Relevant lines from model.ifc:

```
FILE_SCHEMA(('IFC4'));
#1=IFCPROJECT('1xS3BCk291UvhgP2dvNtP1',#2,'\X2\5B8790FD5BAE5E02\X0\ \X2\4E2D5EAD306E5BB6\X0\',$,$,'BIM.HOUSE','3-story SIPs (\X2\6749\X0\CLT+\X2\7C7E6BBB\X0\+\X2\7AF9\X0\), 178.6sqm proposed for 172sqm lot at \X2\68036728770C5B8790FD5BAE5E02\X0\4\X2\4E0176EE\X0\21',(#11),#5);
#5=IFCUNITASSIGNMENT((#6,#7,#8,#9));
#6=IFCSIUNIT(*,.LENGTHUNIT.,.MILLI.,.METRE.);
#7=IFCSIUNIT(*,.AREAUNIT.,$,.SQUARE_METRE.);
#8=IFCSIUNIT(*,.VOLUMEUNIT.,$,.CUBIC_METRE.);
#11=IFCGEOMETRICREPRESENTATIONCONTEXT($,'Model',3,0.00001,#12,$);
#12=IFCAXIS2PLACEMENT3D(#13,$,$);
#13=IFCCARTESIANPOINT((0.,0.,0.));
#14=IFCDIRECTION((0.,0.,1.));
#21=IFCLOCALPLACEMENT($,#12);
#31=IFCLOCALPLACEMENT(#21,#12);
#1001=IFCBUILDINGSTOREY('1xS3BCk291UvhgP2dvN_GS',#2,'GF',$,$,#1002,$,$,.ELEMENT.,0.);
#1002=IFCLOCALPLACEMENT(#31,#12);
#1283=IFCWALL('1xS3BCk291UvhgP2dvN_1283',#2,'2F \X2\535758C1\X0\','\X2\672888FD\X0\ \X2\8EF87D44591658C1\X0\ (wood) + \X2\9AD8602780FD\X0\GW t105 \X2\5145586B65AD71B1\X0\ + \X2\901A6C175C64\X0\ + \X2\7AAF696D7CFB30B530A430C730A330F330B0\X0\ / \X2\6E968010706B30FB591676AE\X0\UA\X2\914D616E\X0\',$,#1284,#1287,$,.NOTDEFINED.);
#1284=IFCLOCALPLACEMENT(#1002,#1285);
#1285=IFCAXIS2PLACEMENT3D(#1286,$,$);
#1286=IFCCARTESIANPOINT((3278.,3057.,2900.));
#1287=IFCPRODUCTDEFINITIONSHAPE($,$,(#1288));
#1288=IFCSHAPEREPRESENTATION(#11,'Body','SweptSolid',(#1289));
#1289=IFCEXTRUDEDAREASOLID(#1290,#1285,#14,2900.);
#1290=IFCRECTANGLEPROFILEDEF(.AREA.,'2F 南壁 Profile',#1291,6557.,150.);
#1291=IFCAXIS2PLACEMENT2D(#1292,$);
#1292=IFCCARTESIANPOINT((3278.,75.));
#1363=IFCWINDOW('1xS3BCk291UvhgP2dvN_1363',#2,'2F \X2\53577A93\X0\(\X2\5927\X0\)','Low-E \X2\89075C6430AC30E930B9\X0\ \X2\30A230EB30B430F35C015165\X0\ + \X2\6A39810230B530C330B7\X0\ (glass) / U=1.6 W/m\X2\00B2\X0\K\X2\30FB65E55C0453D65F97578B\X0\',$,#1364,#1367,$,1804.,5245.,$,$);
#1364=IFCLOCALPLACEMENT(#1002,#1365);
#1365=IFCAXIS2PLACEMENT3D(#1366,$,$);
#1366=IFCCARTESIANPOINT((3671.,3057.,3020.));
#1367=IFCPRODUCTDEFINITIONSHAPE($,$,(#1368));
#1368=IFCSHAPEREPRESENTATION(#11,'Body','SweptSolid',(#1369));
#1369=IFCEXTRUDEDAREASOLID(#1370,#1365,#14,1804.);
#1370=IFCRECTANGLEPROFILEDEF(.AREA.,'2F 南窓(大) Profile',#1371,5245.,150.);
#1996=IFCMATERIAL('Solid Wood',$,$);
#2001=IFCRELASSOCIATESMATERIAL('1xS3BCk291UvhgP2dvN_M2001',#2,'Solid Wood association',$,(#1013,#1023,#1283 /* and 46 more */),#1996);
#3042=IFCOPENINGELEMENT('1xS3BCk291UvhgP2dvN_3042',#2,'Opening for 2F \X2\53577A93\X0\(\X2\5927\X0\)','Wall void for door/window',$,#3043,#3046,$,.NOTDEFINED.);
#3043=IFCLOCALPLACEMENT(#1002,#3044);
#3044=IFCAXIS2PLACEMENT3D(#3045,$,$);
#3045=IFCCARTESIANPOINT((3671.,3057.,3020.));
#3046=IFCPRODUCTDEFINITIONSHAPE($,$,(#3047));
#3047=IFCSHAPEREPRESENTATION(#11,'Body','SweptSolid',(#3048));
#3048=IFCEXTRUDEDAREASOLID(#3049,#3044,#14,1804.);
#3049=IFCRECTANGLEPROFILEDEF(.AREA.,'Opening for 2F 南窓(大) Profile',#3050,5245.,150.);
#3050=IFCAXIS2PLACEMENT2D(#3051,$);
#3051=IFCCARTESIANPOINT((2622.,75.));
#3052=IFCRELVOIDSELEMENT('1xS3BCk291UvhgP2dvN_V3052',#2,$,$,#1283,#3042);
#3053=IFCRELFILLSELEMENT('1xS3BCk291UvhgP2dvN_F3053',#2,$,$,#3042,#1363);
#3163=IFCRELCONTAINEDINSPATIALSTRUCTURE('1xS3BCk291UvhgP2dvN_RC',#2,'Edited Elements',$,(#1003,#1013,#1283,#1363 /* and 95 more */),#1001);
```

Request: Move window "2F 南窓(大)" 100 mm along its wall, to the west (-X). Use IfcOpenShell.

```python
import ifcopenshell
import ifcopenshell.api.geometry
import ifcopenshell.util.placement

model = ifcopenshell.open("model.ifc")

window = model.by_guid("1xS3BCk291UvhgP2dvN_1363")
opening = window.FillsVoids[0].RelatingOpeningElement
wall = opening.VoidsElements[0].RelatingBuildingElement

wall_matrix = ifcopenshell.util.placement.get_local_placement(wall.ObjectPlacement)
shift = wall_matrix[:3, 0] * -100.0
before = ifcopenshell.util.placement.get_local_placement(window.ObjectPlacement)[:3, 3].copy()

# The window is not placed relative to its opening, so move both.
for product in (opening, window):
    matrix = ifcopenshell.util.placement.get_local_placement(product.ObjectPlacement)
    matrix[:3, 3] += shift
    ifcopenshell.api.geometry.edit_object_placement(model, product=product, matrix=matrix, is_si=False)

after = ifcopenshell.util.placement.get_local_placement(window.ObjectPlacement)[:3, 3]
print("window moved by", (after - before).round(3) + 0.0)

model.write("model_rev.ifc")
```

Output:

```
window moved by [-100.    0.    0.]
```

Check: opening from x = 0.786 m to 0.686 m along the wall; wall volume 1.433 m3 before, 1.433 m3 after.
